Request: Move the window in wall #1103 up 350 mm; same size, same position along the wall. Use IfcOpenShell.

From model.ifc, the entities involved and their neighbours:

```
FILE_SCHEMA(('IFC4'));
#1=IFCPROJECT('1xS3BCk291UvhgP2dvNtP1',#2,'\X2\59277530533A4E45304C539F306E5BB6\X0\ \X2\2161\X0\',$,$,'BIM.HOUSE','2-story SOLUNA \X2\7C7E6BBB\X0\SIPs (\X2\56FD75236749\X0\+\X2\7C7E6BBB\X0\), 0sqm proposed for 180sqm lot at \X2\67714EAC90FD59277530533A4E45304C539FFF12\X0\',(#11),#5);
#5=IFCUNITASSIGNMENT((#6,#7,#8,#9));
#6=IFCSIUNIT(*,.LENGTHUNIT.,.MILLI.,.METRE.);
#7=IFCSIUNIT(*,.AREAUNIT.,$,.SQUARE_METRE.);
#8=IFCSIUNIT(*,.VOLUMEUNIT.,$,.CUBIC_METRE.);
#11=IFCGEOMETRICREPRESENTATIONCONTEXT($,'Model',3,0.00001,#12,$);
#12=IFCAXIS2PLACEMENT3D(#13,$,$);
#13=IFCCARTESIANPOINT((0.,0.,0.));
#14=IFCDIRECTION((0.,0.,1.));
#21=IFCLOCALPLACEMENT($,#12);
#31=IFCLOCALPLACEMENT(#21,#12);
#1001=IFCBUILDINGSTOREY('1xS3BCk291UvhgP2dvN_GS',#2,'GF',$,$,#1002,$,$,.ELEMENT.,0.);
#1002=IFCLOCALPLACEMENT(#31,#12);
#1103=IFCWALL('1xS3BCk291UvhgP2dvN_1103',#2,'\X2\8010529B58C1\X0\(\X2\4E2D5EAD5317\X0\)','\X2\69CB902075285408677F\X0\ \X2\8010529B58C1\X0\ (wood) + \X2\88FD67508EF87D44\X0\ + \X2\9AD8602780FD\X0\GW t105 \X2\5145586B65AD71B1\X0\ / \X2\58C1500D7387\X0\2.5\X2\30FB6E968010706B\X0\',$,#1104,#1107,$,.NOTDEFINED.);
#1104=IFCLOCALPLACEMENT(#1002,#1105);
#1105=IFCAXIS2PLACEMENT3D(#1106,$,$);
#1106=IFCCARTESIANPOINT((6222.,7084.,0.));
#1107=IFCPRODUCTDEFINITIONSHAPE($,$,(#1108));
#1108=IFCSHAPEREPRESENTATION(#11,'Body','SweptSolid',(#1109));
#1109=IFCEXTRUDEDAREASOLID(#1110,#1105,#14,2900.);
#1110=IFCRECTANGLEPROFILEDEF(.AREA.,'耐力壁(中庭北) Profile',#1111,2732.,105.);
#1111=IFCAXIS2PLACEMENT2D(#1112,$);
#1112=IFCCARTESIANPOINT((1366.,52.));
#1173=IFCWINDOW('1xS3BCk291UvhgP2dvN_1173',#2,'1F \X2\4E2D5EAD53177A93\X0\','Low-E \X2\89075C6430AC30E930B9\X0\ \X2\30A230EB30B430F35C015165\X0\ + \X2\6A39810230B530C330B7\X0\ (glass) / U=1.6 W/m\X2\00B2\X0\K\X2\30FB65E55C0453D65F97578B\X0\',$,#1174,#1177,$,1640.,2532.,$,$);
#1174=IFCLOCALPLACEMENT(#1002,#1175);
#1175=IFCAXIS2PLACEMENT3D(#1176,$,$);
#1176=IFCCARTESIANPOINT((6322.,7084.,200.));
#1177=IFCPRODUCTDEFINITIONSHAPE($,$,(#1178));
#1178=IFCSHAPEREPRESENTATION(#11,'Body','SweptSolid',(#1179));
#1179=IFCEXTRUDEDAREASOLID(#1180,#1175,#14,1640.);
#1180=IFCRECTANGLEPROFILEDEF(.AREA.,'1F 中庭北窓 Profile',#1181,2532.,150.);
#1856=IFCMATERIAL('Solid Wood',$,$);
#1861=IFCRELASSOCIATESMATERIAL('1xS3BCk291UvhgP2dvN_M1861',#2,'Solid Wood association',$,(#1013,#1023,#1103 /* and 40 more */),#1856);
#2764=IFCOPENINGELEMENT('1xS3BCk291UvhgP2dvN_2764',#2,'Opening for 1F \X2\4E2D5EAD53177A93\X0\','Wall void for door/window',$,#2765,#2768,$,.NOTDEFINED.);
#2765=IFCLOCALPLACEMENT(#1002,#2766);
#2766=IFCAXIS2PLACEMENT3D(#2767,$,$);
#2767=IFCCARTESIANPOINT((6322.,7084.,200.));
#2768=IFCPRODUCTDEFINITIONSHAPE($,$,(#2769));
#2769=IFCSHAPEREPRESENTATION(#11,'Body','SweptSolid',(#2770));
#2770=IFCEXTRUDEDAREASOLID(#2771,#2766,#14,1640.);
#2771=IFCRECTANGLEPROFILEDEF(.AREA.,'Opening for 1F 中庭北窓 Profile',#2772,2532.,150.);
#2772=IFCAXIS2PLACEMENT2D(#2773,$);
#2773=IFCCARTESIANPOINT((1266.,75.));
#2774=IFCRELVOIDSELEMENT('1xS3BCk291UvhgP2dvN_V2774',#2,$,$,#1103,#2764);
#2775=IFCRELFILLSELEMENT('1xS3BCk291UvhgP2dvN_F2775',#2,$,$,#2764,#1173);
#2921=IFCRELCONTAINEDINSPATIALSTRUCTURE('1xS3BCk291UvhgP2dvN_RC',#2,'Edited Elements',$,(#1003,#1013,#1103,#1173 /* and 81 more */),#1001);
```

```python
import numpy as np
import ifcopenshell
import ifcopenshell.api.geometry
import ifcopenshell.util.placement
import ifcopenshell.util.unit

model = ifcopenshell.open("model.ifc")
unit_scale = ifcopenshell.util.unit.calculate_unit_scale(model)

window = model.by_id(1173)
opening = window.FillsVoids[0].RelatingOpeningElement
dz = 0.35 / unit_scale

shift = np.array([0.0, 0.0, dz])
# The window is not placed relative to its opening, so move both.
for product in (opening, window):
    matrix = ifcopenshell.util.placement.get_local_placement(product.ObjectPlacement)
    matrix[:3, 3] += shift
    ifcopenshell.api.geometry.edit_object_placement(model, product=product, matrix=matrix, is_si=False)

print(f"moved by {dz * unit_scale:+.3f} m")

model.write("model_rev.ifc")
```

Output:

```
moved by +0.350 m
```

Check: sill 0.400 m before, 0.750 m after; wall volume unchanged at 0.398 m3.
